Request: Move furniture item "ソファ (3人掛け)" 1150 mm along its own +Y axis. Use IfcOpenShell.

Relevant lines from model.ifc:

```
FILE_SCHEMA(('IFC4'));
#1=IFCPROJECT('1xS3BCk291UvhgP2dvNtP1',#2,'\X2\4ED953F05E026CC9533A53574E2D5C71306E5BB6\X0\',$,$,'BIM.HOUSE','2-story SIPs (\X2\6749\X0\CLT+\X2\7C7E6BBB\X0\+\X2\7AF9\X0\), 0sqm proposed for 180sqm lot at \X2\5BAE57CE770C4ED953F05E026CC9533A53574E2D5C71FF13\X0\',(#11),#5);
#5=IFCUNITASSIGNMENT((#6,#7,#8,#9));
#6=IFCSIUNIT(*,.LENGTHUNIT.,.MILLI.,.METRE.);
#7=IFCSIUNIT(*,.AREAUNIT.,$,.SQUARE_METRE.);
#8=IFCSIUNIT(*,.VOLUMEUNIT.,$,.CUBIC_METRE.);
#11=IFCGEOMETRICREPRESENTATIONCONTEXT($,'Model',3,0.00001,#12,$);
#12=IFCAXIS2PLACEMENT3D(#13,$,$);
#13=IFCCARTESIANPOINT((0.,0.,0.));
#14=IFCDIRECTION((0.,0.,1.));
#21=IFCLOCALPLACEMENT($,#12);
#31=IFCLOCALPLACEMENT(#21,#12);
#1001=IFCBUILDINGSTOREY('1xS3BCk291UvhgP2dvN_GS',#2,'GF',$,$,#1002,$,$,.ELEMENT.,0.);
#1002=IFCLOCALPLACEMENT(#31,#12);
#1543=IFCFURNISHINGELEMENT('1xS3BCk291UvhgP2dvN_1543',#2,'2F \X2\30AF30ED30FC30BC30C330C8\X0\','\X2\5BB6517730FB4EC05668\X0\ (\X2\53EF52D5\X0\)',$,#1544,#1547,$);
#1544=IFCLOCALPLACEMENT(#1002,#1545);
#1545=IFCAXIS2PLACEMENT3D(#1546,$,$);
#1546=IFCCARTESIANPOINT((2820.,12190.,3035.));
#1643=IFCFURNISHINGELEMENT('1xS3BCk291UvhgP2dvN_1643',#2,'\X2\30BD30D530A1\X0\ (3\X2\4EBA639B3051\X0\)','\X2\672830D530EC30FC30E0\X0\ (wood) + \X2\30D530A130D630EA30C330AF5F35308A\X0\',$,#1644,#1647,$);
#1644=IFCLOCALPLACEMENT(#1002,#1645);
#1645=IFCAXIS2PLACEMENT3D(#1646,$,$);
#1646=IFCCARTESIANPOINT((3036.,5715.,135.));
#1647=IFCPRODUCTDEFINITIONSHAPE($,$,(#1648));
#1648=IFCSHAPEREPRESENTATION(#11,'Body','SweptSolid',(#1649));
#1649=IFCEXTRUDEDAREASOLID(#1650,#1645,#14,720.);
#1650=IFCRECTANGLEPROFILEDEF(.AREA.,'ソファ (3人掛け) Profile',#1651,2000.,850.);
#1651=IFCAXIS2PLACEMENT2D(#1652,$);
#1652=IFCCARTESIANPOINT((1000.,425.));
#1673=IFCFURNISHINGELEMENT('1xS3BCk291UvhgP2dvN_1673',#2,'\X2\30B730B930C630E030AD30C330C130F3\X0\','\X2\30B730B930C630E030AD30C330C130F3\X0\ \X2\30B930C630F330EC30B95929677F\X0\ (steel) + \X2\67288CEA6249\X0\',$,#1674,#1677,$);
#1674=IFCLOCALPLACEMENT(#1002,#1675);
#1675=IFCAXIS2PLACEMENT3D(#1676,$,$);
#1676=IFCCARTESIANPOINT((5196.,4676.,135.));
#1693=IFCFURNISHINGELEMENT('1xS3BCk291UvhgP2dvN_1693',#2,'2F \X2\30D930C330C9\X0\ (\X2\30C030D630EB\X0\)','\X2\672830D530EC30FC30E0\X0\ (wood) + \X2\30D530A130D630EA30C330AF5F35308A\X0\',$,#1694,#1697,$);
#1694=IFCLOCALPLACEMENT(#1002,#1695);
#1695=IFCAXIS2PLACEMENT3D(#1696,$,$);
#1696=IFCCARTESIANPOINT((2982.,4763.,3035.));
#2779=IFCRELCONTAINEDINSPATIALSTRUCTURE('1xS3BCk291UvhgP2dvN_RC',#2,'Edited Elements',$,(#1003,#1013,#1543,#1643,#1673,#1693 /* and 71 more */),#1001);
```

```python
import ifcopenshell
import ifcopenshell.api.geometry
import ifcopenshell.util.placement

model = ifcopenshell.open("model.ifc")

item = model.by_guid("1xS3BCk291UvhgP2dvN_1643")
matrix = ifcopenshell.util.placement.get_local_placement(item.ObjectPlacement)
matrix[:3, 3] += matrix[:3, 1] * 1150.0
ifcopenshell.api.geometry.edit_object_placement(model, product=item, matrix=matrix, is_si=False)

print(ifcopenshell.util.placement.get_local_placement(item.ObjectPlacement).round(3) + 0.0)

model.write("model_updated.ifc")
```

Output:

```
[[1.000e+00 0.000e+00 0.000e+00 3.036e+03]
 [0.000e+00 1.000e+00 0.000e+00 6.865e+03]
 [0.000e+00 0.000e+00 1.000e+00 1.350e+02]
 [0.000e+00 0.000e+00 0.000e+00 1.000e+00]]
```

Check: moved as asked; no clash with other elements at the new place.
